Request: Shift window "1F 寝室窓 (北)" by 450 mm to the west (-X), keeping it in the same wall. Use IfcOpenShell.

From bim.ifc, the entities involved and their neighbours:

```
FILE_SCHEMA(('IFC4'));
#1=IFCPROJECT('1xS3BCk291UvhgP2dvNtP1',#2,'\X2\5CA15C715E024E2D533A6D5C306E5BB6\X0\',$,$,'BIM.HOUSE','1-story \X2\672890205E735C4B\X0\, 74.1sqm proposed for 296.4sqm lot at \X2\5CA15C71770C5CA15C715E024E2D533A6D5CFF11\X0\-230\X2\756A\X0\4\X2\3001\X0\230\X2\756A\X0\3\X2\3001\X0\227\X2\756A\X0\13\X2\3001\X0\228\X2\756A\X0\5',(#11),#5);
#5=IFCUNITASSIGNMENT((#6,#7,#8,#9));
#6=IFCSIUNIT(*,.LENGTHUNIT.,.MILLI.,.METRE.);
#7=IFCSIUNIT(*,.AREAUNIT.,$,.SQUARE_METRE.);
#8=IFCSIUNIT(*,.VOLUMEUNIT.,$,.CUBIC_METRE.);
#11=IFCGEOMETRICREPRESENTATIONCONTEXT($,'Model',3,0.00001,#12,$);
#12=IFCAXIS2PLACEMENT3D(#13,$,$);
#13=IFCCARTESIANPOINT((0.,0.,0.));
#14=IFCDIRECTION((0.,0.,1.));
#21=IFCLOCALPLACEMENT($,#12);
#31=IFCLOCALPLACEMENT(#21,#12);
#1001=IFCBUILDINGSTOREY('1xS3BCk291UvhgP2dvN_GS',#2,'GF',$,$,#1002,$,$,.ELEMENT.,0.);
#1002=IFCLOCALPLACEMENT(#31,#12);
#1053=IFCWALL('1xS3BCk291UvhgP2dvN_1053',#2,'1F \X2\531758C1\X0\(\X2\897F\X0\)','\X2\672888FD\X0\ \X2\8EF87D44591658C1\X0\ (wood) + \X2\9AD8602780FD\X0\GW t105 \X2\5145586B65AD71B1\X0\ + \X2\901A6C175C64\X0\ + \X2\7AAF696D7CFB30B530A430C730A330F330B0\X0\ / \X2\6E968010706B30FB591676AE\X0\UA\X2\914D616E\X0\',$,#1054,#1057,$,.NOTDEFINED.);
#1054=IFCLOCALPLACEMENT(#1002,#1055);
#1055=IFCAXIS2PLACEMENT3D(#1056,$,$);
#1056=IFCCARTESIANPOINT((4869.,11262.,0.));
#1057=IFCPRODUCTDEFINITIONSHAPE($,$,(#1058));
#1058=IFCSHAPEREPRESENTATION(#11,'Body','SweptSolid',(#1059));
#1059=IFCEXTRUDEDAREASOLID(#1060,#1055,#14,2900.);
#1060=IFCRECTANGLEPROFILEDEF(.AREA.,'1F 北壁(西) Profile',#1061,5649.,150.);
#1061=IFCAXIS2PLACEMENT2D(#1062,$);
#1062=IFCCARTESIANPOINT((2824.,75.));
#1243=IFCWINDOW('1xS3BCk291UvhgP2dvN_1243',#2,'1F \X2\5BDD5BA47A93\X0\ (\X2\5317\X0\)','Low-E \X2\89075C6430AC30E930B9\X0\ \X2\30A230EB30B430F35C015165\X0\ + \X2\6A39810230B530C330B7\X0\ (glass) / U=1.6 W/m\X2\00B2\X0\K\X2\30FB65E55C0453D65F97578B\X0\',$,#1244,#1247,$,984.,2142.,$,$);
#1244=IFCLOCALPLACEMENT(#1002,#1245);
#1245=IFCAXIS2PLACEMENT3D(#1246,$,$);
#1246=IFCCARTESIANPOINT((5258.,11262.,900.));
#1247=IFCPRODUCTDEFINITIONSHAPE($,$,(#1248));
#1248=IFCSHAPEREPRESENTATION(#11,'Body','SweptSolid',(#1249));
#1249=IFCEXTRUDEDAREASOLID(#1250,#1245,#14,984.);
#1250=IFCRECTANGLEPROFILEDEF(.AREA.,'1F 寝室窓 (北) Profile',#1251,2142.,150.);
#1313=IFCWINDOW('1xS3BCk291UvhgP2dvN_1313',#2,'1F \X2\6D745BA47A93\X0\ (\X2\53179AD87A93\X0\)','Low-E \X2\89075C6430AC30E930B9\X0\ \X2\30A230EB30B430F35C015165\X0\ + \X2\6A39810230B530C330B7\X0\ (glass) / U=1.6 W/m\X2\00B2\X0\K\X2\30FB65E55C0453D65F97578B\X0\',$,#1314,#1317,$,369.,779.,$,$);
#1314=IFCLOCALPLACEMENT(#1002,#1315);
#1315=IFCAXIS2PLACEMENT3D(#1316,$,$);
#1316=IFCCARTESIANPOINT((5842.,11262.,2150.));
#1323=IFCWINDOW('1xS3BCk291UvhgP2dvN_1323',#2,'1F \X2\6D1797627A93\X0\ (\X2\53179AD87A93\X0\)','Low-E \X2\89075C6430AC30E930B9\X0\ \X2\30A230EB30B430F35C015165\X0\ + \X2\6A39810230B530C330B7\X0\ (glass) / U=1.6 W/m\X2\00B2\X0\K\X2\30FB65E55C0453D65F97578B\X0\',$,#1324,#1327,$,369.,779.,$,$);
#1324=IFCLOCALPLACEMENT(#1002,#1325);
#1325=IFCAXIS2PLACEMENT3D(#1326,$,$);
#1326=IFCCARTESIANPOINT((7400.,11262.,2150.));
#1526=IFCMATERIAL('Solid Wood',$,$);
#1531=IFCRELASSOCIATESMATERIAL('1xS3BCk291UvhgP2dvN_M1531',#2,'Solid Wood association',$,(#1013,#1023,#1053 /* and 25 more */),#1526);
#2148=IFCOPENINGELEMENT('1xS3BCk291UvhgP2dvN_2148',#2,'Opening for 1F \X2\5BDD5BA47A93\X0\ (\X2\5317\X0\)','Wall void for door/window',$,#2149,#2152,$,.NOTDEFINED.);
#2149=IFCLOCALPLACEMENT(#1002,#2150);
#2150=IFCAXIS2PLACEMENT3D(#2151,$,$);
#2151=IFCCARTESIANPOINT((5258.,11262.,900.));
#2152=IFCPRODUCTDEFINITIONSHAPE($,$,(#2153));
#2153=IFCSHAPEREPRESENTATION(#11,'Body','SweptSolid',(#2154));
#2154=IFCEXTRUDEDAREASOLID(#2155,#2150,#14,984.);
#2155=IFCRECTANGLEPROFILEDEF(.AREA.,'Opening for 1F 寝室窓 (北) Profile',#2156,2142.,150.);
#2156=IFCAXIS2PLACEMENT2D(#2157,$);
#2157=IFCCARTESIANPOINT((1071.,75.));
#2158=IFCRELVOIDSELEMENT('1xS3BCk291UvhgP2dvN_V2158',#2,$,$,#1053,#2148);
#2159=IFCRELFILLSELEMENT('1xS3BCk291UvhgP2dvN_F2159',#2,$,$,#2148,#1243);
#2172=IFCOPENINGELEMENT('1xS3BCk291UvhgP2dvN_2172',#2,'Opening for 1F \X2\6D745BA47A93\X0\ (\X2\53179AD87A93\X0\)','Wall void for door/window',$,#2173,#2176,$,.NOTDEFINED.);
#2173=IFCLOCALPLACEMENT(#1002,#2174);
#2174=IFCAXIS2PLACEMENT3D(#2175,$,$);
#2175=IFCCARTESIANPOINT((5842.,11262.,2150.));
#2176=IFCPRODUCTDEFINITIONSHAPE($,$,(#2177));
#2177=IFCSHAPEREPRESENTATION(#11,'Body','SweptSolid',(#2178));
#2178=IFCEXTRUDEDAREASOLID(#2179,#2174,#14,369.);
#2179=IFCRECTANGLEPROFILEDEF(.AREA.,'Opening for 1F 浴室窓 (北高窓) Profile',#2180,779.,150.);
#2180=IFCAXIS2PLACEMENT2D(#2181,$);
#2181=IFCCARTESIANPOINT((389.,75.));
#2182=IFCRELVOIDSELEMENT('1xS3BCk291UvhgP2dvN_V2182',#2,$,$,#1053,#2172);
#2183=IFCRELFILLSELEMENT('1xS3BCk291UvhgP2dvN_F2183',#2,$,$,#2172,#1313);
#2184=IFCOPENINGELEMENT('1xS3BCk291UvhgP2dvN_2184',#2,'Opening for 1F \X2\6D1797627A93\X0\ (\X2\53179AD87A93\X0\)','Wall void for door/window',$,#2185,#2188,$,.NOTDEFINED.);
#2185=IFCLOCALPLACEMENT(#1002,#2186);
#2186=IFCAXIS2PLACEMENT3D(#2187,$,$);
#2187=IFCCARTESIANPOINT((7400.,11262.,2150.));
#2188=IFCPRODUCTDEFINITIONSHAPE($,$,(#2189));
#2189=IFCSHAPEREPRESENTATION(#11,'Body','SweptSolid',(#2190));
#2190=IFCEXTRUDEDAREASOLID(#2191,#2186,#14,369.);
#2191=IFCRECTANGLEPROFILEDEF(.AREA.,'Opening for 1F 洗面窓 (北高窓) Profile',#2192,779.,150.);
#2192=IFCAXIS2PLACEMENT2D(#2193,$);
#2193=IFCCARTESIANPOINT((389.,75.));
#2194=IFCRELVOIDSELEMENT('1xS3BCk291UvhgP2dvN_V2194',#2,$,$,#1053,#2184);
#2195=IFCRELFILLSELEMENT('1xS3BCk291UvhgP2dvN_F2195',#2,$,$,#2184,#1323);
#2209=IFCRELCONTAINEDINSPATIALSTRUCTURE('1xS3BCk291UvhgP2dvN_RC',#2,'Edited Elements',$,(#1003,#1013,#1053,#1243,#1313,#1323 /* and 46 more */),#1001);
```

```python
import ifcopenshell
import ifcopenshell.api.geometry
import ifcopenshell.util.placement
import ifcopenshell.util.unit

model = ifcopenshell.open("bim.ifc")
unit_scale = ifcopenshell.util.unit.calculate_unit_scale(model)

window = model.by_guid("1xS3BCk291UvhgP2dvN_1243")
opening = window.FillsVoids[0].RelatingOpeningElement
wall = opening.VoidsElements[0].RelatingBuildingElement

wall_matrix = ifcopenshell.util.placement.get_local_placement(wall.ObjectPlacement)
shift = wall_matrix[:3, 0] * -0.45 / unit_scale
before = ifcopenshell.util.placement.get_local_placement(window.ObjectPlacement)[:3, 3].copy()

# The window is not placed relative to its opening, so move both.
for product in (opening, window):
    matrix = ifcopenshell.util.placement.get_local_placement(product.ObjectPlacement)
    matrix[:3, 3] += shift
    ifcopenshell.api.geometry.edit_object_placement(model, product=product, matrix=matrix, is_si=False)

after = ifcopenshell.util.placement.get_local_placement(window.ObjectPlacement)[:3, 3]
print("window moved by", (after - before).round(3) + 0.0)

model.write("bim_updated.ifc")
```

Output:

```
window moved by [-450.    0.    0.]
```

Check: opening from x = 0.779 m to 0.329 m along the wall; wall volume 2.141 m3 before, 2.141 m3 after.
